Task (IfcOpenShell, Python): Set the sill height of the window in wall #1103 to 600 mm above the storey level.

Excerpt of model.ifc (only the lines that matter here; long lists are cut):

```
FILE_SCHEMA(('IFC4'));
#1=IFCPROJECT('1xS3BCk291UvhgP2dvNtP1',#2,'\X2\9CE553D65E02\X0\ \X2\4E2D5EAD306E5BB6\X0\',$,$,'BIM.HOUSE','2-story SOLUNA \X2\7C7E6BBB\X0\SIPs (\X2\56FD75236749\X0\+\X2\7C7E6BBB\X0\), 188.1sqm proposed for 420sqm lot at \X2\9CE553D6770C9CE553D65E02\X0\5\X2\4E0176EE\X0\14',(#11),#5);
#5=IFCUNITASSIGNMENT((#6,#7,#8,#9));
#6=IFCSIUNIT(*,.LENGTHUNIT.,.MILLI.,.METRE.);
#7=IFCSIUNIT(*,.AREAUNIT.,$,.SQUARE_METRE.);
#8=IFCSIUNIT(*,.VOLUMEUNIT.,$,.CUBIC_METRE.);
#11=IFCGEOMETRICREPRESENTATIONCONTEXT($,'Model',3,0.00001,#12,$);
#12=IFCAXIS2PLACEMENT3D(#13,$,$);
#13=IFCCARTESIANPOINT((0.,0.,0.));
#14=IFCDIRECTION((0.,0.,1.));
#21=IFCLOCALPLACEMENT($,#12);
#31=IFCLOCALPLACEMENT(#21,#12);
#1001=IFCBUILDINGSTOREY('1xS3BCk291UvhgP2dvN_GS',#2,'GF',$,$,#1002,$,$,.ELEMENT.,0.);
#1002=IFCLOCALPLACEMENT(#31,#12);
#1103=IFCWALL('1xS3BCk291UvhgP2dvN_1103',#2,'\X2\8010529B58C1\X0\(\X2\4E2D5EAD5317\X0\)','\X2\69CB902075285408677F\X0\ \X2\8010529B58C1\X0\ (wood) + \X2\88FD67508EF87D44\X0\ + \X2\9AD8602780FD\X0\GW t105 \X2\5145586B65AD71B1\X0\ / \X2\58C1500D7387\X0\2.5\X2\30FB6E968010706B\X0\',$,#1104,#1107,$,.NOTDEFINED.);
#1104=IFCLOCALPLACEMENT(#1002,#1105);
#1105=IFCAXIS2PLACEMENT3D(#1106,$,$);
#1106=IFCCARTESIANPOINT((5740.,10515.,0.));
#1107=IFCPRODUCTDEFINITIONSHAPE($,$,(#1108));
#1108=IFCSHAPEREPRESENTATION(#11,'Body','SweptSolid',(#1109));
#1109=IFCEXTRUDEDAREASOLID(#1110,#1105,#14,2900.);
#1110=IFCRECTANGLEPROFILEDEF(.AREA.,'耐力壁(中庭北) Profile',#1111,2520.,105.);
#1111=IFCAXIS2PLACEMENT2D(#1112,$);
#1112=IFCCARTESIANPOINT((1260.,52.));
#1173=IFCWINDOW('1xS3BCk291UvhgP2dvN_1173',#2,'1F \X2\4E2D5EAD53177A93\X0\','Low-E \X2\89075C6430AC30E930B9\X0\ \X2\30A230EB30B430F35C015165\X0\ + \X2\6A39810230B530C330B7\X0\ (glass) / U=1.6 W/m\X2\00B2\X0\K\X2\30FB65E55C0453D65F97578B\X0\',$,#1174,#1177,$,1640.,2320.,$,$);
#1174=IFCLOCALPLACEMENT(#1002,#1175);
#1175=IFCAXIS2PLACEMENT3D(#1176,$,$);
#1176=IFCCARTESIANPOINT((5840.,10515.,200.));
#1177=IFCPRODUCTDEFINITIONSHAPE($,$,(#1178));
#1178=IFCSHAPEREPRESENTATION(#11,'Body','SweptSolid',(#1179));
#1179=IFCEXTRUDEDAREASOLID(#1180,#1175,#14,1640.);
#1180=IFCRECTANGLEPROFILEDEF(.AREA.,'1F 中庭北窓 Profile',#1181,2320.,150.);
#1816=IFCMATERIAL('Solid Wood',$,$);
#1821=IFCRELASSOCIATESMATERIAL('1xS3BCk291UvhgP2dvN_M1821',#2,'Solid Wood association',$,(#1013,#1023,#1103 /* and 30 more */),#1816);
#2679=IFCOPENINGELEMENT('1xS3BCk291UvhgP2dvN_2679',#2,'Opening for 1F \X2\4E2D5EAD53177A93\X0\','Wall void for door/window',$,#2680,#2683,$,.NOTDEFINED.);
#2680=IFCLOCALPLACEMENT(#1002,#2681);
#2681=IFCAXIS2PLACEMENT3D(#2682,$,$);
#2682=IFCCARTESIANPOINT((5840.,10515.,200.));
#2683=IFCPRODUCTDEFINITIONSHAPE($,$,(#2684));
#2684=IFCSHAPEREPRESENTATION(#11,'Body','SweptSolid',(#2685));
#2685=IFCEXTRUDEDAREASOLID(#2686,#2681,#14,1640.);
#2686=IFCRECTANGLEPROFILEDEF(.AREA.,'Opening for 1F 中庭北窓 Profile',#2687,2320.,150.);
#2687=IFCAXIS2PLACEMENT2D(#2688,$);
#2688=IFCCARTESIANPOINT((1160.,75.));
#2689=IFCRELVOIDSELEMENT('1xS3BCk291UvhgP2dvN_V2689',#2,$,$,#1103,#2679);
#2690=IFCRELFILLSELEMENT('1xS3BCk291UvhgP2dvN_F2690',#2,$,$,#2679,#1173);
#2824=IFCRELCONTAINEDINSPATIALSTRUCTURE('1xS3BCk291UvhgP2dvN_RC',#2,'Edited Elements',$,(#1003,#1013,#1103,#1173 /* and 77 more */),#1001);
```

```python
import numpy as np
import ifcopenshell
import ifcopenshell.api.geometry
import ifcopenshell.geom
import ifcopenshell.util.element
import ifcopenshell.util.placement
import ifcopenshell.util.shape
import ifcopenshell.util.unit

model = ifcopenshell.open("model.ifc")
unit_scale = ifcopenshell.util.unit.calculate_unit_scale(model)

window = model.by_id(1173)
opening = window.FillsVoids[0].RelatingOpeningElement
storey = ifcopenshell.util.element.get_container(window, ifc_class="IfcBuildingStorey")
level = ifcopenshell.util.placement.get_local_placement(storey.ObjectPlacement)[2, 3]

# The opening's origin need not be at the sill, so measure its lowest point.
shape = ifcopenshell.geom.create_shape(ifcopenshell.geom.settings(), opening)
bottom = ifcopenshell.util.shape.get_shape_bottom_elevation(shape, shape.geometry) / unit_scale
dz = level + 0.6 / unit_scale - bottom

shift = np.array([0.0, 0.0, dz])
# The window is not placed relative to its opening, so move both.
for product in (opening, window):
    matrix = ifcopenshell.util.placement.get_local_placement(product.ObjectPlacement)
    matrix[:3, 3] += shift
    ifcopenshell.api.geometry.edit_object_placement(model, product=product, matrix=matrix, is_si=False)

print(f"moved by {dz * unit_scale:+.3f} m")

model.write("model_edited.ifc")
```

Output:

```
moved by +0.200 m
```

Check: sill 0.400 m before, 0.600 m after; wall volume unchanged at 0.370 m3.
